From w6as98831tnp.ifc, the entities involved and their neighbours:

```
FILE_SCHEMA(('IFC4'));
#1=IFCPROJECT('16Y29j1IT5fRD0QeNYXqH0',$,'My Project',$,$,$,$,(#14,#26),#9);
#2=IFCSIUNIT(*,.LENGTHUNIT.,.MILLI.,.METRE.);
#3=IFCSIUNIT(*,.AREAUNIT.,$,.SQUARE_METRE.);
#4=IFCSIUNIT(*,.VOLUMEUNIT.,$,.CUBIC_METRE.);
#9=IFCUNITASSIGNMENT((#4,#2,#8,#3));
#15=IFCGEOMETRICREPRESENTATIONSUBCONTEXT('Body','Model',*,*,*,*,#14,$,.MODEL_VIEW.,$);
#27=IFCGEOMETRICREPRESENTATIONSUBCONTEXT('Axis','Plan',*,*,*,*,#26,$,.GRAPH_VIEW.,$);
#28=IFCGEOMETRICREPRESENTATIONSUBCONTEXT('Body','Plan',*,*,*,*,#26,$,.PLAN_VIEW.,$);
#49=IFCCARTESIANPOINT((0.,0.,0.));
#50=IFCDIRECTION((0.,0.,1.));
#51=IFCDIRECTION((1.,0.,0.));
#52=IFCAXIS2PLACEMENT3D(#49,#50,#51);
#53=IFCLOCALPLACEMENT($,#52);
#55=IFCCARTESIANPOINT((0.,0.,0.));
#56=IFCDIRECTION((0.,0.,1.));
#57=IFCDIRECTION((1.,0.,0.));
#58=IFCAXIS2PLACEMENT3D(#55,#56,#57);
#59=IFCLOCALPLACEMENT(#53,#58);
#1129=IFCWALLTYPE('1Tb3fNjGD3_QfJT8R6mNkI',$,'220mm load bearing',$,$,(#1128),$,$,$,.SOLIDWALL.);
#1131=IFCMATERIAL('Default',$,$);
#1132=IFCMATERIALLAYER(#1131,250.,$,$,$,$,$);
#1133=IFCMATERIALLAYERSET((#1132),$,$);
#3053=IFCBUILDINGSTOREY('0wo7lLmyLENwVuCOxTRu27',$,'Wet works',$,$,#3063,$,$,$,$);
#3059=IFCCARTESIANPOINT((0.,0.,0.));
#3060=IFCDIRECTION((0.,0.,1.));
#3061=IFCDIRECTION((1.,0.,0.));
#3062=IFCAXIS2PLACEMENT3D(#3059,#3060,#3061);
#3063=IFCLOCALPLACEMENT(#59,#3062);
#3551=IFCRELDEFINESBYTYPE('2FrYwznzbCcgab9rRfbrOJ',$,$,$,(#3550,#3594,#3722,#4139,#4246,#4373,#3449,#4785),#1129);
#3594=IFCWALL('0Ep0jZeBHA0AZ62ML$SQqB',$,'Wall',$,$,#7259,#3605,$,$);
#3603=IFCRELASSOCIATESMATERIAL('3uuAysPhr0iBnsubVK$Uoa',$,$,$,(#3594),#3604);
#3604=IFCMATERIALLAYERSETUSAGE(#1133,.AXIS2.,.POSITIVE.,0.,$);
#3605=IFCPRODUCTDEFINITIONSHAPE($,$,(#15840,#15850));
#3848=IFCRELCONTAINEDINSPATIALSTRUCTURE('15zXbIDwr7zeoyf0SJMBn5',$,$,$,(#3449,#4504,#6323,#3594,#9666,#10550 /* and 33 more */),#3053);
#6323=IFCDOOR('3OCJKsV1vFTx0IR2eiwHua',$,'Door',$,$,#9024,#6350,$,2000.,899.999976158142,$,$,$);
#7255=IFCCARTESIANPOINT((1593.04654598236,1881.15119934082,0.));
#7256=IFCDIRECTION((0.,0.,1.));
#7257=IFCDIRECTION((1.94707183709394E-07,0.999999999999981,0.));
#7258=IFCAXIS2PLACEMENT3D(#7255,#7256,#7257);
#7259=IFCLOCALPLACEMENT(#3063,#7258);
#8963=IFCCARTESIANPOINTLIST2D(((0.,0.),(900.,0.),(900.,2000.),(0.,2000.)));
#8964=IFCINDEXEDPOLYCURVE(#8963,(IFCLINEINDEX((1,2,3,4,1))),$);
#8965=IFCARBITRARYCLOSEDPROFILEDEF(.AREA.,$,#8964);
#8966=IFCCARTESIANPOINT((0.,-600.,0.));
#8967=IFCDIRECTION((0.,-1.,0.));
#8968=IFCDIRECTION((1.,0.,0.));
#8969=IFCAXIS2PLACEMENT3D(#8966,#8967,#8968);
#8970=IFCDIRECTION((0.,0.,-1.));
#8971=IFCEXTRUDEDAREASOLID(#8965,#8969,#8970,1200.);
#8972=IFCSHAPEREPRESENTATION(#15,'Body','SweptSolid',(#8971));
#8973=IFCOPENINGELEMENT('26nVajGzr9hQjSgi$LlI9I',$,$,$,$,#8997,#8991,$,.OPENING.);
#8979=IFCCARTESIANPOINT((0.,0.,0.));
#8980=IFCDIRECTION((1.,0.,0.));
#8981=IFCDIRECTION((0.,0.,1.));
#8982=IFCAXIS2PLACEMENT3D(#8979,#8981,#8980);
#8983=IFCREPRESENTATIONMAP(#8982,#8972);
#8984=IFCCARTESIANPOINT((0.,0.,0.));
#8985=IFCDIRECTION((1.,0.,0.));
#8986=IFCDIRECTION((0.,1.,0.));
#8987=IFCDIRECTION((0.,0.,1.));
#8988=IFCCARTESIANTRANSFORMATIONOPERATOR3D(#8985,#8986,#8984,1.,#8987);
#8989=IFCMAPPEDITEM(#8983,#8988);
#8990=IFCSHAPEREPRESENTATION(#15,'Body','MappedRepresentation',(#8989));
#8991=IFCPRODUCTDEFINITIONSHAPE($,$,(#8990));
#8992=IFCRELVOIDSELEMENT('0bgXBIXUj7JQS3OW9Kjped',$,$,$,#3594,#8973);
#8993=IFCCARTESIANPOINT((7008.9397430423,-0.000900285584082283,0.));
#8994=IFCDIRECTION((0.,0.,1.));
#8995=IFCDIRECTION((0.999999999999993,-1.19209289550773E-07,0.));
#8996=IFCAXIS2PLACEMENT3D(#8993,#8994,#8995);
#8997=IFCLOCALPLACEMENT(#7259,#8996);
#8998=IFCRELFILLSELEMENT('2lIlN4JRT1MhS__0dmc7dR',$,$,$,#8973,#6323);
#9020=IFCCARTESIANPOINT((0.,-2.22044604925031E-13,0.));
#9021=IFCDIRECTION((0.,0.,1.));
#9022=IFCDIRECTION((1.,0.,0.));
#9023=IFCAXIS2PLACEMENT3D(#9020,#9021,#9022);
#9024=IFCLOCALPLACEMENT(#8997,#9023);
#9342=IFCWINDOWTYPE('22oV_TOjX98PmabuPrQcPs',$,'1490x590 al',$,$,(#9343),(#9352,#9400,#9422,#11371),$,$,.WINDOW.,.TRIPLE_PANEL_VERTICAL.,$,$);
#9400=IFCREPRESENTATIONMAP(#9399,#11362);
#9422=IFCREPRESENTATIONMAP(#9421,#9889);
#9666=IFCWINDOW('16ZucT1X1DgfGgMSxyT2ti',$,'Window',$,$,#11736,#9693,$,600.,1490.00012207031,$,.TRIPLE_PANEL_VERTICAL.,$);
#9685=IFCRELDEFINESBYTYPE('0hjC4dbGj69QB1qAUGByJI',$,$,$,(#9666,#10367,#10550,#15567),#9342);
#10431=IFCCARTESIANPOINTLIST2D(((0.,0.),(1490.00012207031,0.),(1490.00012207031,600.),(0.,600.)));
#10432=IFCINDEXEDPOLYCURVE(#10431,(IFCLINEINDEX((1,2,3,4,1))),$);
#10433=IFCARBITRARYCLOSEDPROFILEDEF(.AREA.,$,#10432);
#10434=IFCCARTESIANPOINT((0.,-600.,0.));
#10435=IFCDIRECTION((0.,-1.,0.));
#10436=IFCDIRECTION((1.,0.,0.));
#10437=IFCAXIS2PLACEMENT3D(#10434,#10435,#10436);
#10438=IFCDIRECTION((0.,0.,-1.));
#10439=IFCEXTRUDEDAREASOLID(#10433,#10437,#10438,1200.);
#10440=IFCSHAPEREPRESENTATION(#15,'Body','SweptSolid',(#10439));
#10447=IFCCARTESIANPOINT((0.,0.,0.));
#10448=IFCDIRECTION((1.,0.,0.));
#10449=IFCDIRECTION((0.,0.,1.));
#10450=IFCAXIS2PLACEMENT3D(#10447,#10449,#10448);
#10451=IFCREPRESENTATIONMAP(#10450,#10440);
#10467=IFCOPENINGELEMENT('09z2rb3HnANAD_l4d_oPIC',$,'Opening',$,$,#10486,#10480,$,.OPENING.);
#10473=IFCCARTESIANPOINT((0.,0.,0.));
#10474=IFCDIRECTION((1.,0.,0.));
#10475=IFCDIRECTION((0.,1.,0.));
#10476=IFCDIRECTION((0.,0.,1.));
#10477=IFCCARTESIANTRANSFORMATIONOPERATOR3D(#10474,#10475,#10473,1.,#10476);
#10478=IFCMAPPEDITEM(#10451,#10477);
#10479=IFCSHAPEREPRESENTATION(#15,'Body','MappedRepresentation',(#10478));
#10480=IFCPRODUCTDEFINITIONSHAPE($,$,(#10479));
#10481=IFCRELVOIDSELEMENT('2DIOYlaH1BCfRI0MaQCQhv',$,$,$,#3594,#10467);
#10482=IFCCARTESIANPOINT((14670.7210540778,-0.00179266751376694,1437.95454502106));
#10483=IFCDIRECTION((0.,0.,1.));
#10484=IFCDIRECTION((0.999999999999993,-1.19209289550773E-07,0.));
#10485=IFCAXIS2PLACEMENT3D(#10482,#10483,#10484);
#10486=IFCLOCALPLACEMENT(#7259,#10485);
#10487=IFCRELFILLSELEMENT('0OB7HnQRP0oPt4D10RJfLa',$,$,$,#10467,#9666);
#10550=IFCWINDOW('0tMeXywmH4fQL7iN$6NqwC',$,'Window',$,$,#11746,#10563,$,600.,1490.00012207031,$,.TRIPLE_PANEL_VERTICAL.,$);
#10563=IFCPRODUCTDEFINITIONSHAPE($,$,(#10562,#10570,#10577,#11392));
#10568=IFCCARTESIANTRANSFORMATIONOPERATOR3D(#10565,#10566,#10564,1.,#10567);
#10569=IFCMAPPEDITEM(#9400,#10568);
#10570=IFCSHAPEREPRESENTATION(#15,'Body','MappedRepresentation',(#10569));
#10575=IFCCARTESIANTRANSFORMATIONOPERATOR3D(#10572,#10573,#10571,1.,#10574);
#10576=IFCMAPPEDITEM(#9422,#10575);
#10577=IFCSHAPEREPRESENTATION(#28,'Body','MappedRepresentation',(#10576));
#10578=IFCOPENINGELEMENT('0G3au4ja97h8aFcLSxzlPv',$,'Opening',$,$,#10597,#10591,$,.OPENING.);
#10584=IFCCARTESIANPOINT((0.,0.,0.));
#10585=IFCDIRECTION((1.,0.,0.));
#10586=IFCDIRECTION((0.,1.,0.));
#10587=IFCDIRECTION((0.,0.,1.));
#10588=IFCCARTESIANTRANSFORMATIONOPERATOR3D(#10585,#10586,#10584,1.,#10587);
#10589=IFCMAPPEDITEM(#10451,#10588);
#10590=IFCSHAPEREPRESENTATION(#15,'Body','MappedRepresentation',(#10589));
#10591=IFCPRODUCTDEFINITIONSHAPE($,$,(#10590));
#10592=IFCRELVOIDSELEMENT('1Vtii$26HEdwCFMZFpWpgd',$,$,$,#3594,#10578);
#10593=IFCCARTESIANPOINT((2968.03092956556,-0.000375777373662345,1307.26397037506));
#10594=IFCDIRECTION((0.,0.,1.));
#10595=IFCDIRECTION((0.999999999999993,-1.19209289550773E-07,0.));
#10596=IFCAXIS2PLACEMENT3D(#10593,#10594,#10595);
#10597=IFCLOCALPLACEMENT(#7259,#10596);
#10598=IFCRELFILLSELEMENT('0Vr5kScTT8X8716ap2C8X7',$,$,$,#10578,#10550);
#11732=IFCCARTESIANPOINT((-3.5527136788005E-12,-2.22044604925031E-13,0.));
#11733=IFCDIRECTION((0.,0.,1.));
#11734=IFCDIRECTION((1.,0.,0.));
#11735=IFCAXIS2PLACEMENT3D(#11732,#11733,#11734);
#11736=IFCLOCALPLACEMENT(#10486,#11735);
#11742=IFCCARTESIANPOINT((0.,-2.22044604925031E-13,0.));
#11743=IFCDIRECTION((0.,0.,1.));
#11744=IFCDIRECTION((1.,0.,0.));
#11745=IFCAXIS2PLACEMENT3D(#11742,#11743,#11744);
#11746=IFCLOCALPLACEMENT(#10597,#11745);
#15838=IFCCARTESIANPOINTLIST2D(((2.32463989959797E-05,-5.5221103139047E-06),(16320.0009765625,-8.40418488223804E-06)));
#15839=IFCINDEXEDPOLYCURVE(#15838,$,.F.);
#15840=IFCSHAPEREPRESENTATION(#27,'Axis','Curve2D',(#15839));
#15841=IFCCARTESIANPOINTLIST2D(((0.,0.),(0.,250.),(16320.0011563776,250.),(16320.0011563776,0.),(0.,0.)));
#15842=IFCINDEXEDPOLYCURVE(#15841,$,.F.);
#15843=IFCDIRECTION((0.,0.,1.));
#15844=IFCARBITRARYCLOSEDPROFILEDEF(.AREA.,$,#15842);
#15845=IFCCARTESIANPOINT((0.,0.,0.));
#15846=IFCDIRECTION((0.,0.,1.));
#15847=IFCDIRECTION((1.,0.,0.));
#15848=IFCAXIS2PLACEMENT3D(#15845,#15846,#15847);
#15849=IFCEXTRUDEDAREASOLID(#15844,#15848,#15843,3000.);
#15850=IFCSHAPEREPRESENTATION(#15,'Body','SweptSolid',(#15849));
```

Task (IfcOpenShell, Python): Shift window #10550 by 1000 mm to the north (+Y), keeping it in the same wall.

```python
import ifcopenshell
import ifcopenshell.api.geometry
import ifcopenshell.util.placement

model = ifcopenshell.open("w6as98831tnp.ifc")

window = model.by_guid("0tMeXywmH4fQL7iN$6NqwC")
opening = window.FillsVoids[0].RelatingOpeningElement
wall = opening.VoidsElements[0].RelatingBuildingElement

wall_matrix = ifcopenshell.util.placement.get_local_placement(wall.ObjectPlacement)
shift = wall_matrix[:3, 0] * 1000.0
before = ifcopenshell.util.placement.get_local_placement(window.ObjectPlacement)[:3, 3].copy()

# The window is placed relative to its opening, so it follows when the opening moves.
matrix = ifcopenshell.util.placement.get_local_placement(opening.ObjectPlacement)
matrix[:3, 3] += shift
ifcopenshell.api.geometry.edit_object_placement(
    model, product=opening, matrix=matrix, is_si=False, should_transform_children=True
)

after = ifcopenshell.util.placement.get_local_placement(window.ObjectPlacement)[:3, 3]
print("window moved by", (after - before).round(3) + 0.0)

model.write("w6as98831tnp_rev.ifc")
```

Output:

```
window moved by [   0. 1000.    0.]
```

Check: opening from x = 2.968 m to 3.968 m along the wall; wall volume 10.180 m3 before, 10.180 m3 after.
